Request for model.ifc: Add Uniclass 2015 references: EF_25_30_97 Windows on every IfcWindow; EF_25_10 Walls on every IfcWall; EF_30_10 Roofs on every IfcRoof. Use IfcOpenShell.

First a look at what the model holds.

```python
import ifcopenshell

model = ifcopenshell.open("model.ifc")
print(model.schema)
print("classifications:", [c.Name for c in model.by_type("IfcClassification")])
for ifc_class in ("IfcDoor", "IfcRoof", "IfcStair", "IfcWall", "IfcWindow"):
    print(ifc_class, len(model.by_type(ifc_class)))
```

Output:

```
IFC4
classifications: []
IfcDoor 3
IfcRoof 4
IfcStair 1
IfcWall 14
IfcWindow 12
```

```python
import ifcopenshell
import ifcopenshell.api.classification

model = ifcopenshell.open("model.ifc")

system = ifcopenshell.api.classification.add_classification(model, classification="Uniclass 2015")

codes = {
    "IfcWindow": ("EF_25_30_97", "Windows"),
    "IfcWall": ("EF_25_10", "Walls"),
    "IfcRoof": ("EF_30_10", "Roofs"),
}
for ifc_class, (code, name) in codes.items():
    products = model.by_type(ifc_class)
    ifcopenshell.api.classification.add_reference(
        model, products=products, classification=system, identification=code, name=name
    )
    print(code, len(products))

model.write("model_rev.ifc")
```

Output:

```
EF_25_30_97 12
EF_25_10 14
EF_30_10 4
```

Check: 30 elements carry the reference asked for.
